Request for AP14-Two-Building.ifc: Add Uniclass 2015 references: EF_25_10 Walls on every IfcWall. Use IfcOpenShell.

First a look at what the model holds.

```python
import ifcopenshell

model = ifcopenshell.open("AP14-Two-Building.ifc")
print(model.schema)
print("classifications:", [c.Name for c in model.by_type("IfcClassification")])
for ifc_class in ("IfcDoor", "IfcRoof", "IfcStair", "IfcWall", "IfcWindow"):
    print(ifc_class, len(model.by_type(ifc_class)))
```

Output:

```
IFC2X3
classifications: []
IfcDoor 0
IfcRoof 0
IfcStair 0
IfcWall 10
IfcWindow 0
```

```python
import ifcopenshell
import ifcopenshell.api.classification

model = ifcopenshell.open("AP14-Two-Building.ifc")

# IFC2X3 requires Source and Edition and has no link from the project to the system.
system = model.create_entity("IfcClassification", Source="NBS", Edition="2015", Name="Uniclass 2015")

codes = {
    "IfcWall": ("EF_25_10", "Walls"),
}
for ifc_class, (code, name) in codes.items():
    products = model.by_type(ifc_class)
    ifcopenshell.api.classification.add_reference(
        model, products=products, classification=system, identification=code, name=name
    )
    print(code, len(products))

model.write("AP14-Two-Building_rev.ifc")
```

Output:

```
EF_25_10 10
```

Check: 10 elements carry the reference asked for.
